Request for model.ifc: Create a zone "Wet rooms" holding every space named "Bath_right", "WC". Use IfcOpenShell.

First a look at what the model holds.

```python
import ifcopenshell

model = ifcopenshell.open("model.ifc")
print(model.schema)
seen = {}
for space in model.by_type("IfcSpace"):
    seen[space.LongName] = seen.get(space.LongName, 0) + 1
for name, count in sorted(seen.items(), key=str):
    print(count, "x", name)
print("zones:", [z.Name for z in model.by_type("IfcZone")][:20])
```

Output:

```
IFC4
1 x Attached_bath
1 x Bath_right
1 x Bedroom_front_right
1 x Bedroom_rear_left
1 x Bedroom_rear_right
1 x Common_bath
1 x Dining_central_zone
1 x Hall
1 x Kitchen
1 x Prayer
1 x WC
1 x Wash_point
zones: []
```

```python
import ifcopenshell
import ifcopenshell.api.group
import ifcopenshell.api.root

model = ifcopenshell.open("model.ifc")

names = {"Bath_right", "WC"}
spaces = [s for s in model.by_type("IfcSpace") if s.LongName in names]

zone = ifcopenshell.api.root.create_entity(model, ifc_class="IfcZone", name="Wet rooms")
ifcopenshell.api.group.assign_group(model, products=spaces, group=zone)
print(len(spaces), "spaces in", zone.Name)

model.write("model_v2.ifc")
```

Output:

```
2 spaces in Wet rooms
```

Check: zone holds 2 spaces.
